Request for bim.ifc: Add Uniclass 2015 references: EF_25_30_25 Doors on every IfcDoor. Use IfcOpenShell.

First a look at what the model holds.

```python
import ifcopenshell

model = ifcopenshell.open("bim.ifc")
print(model.schema)
print("classifications:", [c.Name for c in model.by_type("IfcClassification")])
for ifc_class in ("IfcDoor", "IfcRoof", "IfcStair", "IfcWall", "IfcWindow"):
    print(ifc_class, len(model.by_type(ifc_class)))
```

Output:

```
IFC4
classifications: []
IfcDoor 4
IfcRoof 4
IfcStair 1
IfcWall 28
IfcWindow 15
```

```python
import ifcopenshell
import ifcopenshell.api.classification

model = ifcopenshell.open("bim.ifc")

system = ifcopenshell.api.classification.add_classification(model, classification="Uniclass 2015")

codes = {
    "IfcDoor": ("EF_25_30_25", "Doors"),
}
for ifc_class, (code, name) in codes.items():
    products = model.by_type(ifc_class)
    ifcopenshell.api.classification.add_reference(
        model, products=products, classification=system, identification=code, name=name
    )
    print(code, len(products))

model.write("bim_edited.ifc")
```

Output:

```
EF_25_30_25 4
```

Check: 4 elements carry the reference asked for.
